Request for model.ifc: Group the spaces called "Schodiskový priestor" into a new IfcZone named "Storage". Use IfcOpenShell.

First a look at what the model holds.

```python
import ifcopenshell

model = ifcopenshell.open("model.ifc")
print(model.schema)
seen = {}
for space in model.by_type("IfcSpace"):
    seen[space.LongName] = seen.get(space.LongName, 0) + 1
for name, count in sorted(seen.items(), key=str):
    print(count, "x", name)
print("zones:", [z.Name for z in model.by_type("IfcZone")][:20])
```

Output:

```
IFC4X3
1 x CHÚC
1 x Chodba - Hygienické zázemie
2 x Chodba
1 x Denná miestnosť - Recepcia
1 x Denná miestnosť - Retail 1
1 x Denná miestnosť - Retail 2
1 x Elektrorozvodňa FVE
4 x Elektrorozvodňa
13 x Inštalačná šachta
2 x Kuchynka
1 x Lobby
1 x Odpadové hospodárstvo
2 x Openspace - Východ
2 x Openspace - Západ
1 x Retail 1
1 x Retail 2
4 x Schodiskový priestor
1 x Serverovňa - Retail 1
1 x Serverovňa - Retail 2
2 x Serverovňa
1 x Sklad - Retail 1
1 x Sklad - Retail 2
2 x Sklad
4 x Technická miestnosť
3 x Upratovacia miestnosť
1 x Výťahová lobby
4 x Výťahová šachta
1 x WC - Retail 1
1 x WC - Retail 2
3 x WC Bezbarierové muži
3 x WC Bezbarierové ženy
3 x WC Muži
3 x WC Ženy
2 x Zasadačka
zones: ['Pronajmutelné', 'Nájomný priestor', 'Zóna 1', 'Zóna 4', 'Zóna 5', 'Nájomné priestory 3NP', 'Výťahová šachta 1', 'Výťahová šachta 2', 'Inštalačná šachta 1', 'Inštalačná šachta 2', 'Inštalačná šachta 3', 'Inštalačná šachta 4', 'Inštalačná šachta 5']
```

```python
import ifcopenshell
import ifcopenshell.api.group
import ifcopenshell.api.root

model = ifcopenshell.open("model.ifc")

names = {"Schodiskový priestor"}
spaces = [s for s in model.by_type("IfcSpace") if s.LongName in names]

zone = ifcopenshell.api.root.create_entity(model, ifc_class="IfcZone", name="Storage")
ifcopenshell.api.group.assign_group(model, products=spaces, group=zone)
print(len(spaces), "spaces in", zone.Name)

model.write("model_edited.ifc")
```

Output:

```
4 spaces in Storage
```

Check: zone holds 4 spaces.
